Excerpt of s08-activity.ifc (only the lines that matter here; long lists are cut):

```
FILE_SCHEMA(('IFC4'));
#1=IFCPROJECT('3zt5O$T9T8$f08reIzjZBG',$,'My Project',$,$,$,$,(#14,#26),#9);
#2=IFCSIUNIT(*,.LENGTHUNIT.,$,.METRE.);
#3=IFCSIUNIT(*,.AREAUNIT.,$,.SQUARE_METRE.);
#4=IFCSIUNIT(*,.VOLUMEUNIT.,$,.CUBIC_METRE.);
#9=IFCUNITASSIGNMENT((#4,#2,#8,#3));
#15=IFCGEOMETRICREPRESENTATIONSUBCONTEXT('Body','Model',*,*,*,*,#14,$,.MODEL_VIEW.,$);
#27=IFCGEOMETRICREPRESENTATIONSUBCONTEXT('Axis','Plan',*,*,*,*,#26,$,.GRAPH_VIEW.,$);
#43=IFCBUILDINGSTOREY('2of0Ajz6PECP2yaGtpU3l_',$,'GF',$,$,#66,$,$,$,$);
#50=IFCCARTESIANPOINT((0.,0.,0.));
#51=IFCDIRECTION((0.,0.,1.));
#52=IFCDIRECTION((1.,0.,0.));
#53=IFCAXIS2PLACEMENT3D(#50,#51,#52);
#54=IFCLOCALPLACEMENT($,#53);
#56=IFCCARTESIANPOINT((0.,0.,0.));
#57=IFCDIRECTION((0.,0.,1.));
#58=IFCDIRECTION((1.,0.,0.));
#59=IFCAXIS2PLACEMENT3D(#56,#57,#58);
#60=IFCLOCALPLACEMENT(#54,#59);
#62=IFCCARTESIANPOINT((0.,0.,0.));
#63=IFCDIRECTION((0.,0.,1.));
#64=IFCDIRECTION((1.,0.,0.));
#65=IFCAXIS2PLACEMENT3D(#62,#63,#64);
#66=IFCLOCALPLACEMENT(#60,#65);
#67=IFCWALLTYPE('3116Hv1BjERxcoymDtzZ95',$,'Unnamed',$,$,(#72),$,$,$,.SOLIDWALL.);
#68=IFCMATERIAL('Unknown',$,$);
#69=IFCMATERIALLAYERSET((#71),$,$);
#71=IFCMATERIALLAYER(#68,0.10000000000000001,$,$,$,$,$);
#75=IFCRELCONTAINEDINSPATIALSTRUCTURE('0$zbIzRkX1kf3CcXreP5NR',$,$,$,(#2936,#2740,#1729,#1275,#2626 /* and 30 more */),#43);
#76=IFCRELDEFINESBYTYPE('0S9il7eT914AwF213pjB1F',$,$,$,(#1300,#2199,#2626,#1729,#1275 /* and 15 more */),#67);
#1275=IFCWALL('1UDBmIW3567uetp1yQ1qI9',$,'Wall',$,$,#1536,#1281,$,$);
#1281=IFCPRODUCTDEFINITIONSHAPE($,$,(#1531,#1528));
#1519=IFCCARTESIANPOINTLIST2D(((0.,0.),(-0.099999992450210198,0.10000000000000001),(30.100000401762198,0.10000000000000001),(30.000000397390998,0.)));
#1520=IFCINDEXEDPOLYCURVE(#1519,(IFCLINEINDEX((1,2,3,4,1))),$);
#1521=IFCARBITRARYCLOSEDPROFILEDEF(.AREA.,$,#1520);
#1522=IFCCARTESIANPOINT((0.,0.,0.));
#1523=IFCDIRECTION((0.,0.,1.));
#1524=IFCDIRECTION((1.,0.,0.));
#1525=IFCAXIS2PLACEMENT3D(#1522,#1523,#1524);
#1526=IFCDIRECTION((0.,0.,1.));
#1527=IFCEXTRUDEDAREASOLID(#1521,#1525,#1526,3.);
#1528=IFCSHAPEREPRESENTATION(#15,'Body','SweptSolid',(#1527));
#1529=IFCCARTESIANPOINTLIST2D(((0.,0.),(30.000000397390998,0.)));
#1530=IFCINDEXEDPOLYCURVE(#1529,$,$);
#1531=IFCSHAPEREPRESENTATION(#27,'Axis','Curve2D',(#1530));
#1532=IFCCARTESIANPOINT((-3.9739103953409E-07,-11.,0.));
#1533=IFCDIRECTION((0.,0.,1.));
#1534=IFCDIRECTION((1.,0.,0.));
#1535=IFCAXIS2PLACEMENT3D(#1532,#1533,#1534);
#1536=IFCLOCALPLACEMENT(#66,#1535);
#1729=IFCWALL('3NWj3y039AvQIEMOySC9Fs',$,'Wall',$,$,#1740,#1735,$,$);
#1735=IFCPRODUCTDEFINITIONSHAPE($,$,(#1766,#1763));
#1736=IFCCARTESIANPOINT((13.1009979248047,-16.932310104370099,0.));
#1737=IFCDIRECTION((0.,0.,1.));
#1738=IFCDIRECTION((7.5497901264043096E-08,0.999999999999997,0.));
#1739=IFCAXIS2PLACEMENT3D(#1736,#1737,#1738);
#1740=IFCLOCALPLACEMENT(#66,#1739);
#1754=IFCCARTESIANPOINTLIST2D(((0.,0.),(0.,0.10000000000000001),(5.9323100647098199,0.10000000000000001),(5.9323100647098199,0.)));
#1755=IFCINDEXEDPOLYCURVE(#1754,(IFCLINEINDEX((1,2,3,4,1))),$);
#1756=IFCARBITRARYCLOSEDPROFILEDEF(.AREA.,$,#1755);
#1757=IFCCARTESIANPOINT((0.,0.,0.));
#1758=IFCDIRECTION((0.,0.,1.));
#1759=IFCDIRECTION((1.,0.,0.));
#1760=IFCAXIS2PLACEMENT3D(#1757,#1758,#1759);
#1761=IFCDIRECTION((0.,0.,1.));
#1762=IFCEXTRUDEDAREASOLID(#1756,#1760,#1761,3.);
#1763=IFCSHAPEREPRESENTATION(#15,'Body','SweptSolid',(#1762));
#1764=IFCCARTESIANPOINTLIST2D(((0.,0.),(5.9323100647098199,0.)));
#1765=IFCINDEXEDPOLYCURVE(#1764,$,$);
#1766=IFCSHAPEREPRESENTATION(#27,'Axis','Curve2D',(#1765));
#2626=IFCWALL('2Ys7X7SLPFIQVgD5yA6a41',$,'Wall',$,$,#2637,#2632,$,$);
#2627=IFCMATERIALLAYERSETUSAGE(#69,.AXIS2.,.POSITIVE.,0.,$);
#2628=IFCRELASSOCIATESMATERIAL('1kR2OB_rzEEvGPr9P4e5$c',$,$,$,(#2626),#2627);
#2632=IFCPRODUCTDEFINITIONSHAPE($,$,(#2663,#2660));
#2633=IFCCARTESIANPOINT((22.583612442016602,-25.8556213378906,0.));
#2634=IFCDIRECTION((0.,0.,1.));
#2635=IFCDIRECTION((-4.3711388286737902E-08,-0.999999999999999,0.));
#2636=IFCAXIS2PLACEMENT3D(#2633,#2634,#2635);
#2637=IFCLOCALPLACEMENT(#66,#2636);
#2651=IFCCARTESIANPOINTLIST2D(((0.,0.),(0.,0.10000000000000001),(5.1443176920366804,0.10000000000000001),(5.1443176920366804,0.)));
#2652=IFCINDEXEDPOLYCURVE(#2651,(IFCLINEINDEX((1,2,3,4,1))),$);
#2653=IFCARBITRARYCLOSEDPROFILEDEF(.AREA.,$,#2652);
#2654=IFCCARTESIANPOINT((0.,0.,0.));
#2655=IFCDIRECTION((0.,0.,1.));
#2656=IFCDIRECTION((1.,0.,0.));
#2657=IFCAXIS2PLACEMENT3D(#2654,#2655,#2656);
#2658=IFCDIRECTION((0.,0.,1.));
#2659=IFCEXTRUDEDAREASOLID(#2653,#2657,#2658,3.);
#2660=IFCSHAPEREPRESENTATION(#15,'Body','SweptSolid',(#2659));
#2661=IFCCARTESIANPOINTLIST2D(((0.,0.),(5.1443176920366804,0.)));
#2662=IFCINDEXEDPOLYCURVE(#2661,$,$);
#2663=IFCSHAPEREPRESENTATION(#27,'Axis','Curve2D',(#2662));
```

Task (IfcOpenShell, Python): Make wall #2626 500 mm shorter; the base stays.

```python
import ifcopenshell
import ifcopenshell.geom
import ifcopenshell.util.representation
import ifcopenshell.util.shape
import ifcopenshell.util.unit

model = ifcopenshell.open("s08-activity.ifc")
unit_scale = ifcopenshell.util.unit.calculate_unit_scale(model)
settings = ifcopenshell.geom.settings()


def volume(element):
    """Net volume in cubic metres, openings subtracted."""
    shape = ifcopenshell.geom.create_shape(settings, element)
    return ifcopenshell.util.shape.get_volume(shape.geometry)


wall = model.by_guid("2Ys7X7SLPFIQVgD5yA6a41")
before = volume(wall)

body = ifcopenshell.util.representation.get_representation(wall, "Model", "Body")
solid = body.Items[0]
old_height = solid.Depth
solid.Depth -= 0.5 / unit_scale
after = volume(wall)

print(f"height {old_height:g} -> {solid.Depth:g}, volume {before:.3f} -> {after:.3f} m3")

model.write("s08-activity_v2.ifc")
```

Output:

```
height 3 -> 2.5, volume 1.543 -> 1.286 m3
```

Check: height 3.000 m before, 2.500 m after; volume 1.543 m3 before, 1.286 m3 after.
